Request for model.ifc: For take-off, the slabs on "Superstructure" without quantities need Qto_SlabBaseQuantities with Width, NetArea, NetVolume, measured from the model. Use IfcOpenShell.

First a look at what the model holds.

```python
import ifcopenshell
import ifcopenshell.util.element
import ifcopenshell.util.unit

model = ifcopenshell.open("model.ifc")
print(model.schema)
for unit_type in ("LENGTHUNIT", "AREAUNIT", "VOLUMEUNIT"):
    print(unit_type, ifcopenshell.util.unit.calculate_unit_scale(model, unit_type))
storey = next(s for s in model.by_type("IfcBuildingStorey") if s.Name == "Superstructure")
slabs = [e for e in ifcopenshell.util.element.get_decomposition(storey) if e.is_a("IfcSlab")]
for e in sorted(slabs, key=lambda e: e.id()):
    print(e.id(), e.is_a(), e.Name, list(ifcopenshell.util.element.get_psets(e, qtos_only=True)), sep=" | ")
```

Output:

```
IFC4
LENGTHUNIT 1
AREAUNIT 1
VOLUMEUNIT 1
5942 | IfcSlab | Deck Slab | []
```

```python
import ifcopenshell
import ifcopenshell.api.pset
import ifcopenshell.geom
import ifcopenshell.util.element
import ifcopenshell.util.shape
import ifcopenshell.util.unit

model = ifcopenshell.open("model.ifc")
unit_scale = ifcopenshell.util.unit.calculate_unit_scale(model)
area_scale = ifcopenshell.util.unit.calculate_unit_scale(model, "AREAUNIT")
volume_scale = ifcopenshell.util.unit.calculate_unit_scale(model, "VOLUMEUNIT")
settings = ifcopenshell.geom.settings()

storey = next(s for s in model.by_type("IfcBuildingStorey") if s.Name == "Superstructure")
slabs = [e for e in ifcopenshell.util.element.get_decomposition(storey) if e.is_a("IfcSlab")]

for e in sorted(slabs, key=lambda e: e.id()):
    if ifcopenshell.util.element.get_psets(e, qtos_only=True, should_inherit=False):
        continue
    # Geometry comes back in metres, in the element's own axes.
    shape = ifcopenshell.geom.create_shape(settings, e)
    values = {
        "Width": ifcopenshell.util.shape.get_z(shape.geometry) / unit_scale,
        "NetArea": ifcopenshell.util.shape.get_footprint_area(shape.geometry) / area_scale,
        "NetVolume": ifcopenshell.util.shape.get_volume(shape.geometry) / volume_scale,
    }
    qto = ifcopenshell.api.pset.add_qto(model, product=e, name="Qto_SlabBaseQuantities")
    ifcopenshell.api.pset.edit_qto(model, qto=qto, properties=values)
    print(e.id(), {k: round(v, 3) for k, v in values.items()})

model.write("model_updated.ifc")
```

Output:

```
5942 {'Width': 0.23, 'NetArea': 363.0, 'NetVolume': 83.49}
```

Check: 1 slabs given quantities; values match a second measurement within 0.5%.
